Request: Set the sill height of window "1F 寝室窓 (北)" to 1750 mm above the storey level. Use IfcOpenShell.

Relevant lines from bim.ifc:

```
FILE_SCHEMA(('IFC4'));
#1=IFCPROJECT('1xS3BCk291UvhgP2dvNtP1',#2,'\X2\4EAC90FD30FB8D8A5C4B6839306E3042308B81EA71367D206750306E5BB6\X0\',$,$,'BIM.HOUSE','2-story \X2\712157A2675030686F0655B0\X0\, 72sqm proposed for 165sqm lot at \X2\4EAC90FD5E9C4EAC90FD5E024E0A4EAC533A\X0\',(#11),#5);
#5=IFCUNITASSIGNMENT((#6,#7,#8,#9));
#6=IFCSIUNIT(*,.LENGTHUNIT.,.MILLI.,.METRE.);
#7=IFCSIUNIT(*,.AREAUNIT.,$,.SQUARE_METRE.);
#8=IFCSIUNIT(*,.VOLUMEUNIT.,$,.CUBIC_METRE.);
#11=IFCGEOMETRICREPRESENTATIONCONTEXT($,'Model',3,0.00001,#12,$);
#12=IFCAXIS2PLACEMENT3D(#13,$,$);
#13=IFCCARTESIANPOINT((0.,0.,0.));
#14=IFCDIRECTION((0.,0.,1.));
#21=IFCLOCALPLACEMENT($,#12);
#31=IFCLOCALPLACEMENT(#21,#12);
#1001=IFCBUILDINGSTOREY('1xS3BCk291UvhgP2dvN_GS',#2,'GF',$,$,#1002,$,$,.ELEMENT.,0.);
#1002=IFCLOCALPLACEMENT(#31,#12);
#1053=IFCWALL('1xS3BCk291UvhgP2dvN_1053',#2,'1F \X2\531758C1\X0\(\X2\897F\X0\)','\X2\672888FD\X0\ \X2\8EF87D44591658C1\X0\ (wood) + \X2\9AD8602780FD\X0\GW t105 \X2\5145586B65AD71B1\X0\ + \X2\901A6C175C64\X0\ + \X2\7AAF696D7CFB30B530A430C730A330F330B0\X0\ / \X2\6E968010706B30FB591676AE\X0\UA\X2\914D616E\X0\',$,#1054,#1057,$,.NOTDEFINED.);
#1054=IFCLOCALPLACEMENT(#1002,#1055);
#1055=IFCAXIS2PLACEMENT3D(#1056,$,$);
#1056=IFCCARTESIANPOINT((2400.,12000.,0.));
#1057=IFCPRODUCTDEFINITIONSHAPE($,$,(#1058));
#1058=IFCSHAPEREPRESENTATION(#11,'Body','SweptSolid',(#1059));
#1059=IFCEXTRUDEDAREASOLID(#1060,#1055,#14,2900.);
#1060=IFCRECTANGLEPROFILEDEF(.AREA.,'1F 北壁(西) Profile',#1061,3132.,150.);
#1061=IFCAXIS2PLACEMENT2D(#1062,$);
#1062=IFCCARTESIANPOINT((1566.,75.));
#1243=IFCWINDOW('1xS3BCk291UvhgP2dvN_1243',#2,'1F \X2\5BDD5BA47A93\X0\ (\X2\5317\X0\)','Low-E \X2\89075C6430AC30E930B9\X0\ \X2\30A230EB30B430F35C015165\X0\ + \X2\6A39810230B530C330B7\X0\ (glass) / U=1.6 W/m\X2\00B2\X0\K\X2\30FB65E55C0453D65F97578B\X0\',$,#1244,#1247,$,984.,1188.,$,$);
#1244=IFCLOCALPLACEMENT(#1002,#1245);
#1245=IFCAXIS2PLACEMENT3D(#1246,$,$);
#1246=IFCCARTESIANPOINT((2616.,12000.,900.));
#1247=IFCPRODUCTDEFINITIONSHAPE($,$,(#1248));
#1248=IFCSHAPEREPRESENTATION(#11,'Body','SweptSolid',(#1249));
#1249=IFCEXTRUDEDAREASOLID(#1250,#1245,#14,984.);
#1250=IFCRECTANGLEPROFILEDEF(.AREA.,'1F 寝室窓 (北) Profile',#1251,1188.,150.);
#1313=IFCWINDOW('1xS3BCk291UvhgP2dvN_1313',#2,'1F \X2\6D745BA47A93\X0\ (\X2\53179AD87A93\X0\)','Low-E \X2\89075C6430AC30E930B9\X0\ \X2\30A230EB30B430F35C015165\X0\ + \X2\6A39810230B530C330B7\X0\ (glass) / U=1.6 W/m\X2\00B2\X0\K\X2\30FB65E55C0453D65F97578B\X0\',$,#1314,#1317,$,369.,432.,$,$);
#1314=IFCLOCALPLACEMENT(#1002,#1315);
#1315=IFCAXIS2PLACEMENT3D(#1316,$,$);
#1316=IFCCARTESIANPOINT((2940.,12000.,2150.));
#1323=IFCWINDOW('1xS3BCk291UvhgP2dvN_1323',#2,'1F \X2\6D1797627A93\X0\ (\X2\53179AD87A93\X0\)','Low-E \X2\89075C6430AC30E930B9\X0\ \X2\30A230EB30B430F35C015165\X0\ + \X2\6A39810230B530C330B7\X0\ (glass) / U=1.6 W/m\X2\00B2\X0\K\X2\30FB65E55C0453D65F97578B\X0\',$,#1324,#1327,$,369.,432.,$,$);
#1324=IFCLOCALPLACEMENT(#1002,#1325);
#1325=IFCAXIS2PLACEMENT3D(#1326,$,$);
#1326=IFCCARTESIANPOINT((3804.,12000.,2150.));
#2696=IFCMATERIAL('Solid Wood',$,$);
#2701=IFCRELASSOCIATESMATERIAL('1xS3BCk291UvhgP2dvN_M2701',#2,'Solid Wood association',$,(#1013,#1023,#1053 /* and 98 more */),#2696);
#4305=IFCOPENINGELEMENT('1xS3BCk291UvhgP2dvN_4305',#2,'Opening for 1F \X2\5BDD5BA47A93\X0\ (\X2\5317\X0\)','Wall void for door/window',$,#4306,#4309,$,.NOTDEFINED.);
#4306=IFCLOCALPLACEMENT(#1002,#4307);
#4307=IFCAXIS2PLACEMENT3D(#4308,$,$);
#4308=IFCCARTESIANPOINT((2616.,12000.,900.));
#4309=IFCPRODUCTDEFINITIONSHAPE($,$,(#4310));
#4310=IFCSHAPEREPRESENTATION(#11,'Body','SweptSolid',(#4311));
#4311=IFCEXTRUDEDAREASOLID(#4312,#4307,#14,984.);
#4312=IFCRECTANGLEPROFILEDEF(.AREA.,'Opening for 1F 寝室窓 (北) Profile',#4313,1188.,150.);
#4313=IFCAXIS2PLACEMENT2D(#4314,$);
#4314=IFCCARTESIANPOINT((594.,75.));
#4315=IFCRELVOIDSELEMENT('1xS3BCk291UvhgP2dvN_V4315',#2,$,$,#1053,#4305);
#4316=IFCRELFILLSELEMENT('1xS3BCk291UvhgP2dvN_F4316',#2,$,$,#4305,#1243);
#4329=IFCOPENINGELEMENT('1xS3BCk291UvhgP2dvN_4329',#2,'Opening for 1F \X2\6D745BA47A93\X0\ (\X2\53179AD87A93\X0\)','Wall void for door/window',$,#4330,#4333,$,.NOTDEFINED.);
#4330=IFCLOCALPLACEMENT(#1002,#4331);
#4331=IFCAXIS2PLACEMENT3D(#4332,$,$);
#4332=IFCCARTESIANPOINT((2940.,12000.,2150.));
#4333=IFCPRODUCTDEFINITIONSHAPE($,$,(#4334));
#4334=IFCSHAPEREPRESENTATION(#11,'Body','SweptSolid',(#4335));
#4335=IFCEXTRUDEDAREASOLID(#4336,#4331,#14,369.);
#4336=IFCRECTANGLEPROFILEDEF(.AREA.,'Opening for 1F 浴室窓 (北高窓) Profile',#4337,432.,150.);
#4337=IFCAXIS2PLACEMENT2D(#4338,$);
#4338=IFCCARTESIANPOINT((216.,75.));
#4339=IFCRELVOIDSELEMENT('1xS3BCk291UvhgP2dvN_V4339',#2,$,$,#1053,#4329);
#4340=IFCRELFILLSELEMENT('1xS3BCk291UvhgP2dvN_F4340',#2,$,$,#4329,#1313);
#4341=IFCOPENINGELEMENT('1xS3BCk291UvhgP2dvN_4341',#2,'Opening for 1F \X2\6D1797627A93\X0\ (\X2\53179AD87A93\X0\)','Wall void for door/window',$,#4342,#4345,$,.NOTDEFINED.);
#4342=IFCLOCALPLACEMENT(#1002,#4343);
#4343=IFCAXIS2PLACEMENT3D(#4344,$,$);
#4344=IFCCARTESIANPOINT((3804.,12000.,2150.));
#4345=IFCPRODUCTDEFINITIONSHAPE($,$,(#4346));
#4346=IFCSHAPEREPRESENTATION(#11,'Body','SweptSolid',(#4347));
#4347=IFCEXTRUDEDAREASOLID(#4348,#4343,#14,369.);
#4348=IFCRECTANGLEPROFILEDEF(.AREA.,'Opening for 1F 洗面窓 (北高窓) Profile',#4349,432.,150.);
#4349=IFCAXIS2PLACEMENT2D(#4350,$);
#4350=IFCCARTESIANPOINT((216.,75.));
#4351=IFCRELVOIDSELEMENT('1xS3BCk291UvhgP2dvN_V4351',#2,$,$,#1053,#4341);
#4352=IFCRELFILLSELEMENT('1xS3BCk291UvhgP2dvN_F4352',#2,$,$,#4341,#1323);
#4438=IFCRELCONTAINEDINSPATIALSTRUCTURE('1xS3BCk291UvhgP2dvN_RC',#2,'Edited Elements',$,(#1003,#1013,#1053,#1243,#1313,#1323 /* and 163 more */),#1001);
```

```python
import numpy as np
import ifcopenshell
import ifcopenshell.api.geometry
import ifcopenshell.geom
import ifcopenshell.util.element
import ifcopenshell.util.placement
import ifcopenshell.util.shape
import ifcopenshell.util.unit

model = ifcopenshell.open("bim.ifc")
unit_scale = ifcopenshell.util.unit.calculate_unit_scale(model)

window = model.by_guid("1xS3BCk291UvhgP2dvN_1243")
opening = window.FillsVoids[0].RelatingOpeningElement
storey = ifcopenshell.util.element.get_container(window, ifc_class="IfcBuildingStorey")
level = ifcopenshell.util.placement.get_local_placement(storey.ObjectPlacement)[2, 3]

# The opening's origin need not be at the sill, so measure its lowest point.
shape = ifcopenshell.geom.create_shape(ifcopenshell.geom.settings(), opening)
bottom = ifcopenshell.util.shape.get_shape_bottom_elevation(shape, shape.geometry) / unit_scale
dz = level + 1.75 / unit_scale - bottom

shift = np.array([0.0, 0.0, dz])
# The window is not placed relative to its opening, so move both.
for product in (opening, window):
    matrix = ifcopenshell.util.placement.get_local_placement(product.ObjectPlacement)
    matrix[:3, 3] += shift
    ifcopenshell.api.geometry.edit_object_placement(model, product=product, matrix=matrix, is_si=False)

print(f"moved by {dz * unit_scale:+.3f} m")

model.write("bim_v2.ifc")
```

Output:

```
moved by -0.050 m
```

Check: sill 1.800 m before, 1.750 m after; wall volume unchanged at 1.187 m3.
